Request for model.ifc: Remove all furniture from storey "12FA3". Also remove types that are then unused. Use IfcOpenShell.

First a look at what the model holds.

```python
import ifcopenshell
import ifcopenshell.util.element

model = ifcopenshell.open("model.ifc")
print(model.schema)
storey = next(s for s in model.by_type("IfcBuildingStorey") if s.Name == "12FA3")
furniture = [e for e in ifcopenshell.util.element.get_decomposition(storey) if e.is_a("IfcFurnishingElement")]
seen = {}
for e in furniture:
    element_type = ifcopenshell.util.element.get_type(e)
    name = element_type.Name if element_type not in (None, e) else None
    seen[name] = seen.get(name, 0) + 1
for name, count in sorted(seen.items(), key=str):
    print(count, "x", name)
```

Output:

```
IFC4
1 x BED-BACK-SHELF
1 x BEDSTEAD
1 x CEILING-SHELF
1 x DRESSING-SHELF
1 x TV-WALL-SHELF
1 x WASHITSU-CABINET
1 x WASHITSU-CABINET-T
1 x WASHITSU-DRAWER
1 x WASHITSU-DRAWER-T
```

```python
import ifcopenshell
import ifcopenshell.api.root
import ifcopenshell.util.element

model = ifcopenshell.open("model.ifc")

storey = next(s for s in model.by_type("IfcBuildingStorey") if s.Name == "12FA3")
furniture = [e for e in ifcopenshell.util.element.get_decomposition(storey) if e.is_a("IfcFurnishingElement")]
types = {ifcopenshell.util.element.get_type(e) for e in furniture} - {None, *furniture}

for e in furniture:
    ifcopenshell.api.root.remove_product(model, product=e)
print(len(furniture), "removed")

unused = [t for t in types if not ifcopenshell.util.element.get_types(t)]
for t in unused:
    ifcopenshell.api.root.remove_product(model, product=t)
print(len(unused), "unused types removed")

model.write("model_rev.ifc")
```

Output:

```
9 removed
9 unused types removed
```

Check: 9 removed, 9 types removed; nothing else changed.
